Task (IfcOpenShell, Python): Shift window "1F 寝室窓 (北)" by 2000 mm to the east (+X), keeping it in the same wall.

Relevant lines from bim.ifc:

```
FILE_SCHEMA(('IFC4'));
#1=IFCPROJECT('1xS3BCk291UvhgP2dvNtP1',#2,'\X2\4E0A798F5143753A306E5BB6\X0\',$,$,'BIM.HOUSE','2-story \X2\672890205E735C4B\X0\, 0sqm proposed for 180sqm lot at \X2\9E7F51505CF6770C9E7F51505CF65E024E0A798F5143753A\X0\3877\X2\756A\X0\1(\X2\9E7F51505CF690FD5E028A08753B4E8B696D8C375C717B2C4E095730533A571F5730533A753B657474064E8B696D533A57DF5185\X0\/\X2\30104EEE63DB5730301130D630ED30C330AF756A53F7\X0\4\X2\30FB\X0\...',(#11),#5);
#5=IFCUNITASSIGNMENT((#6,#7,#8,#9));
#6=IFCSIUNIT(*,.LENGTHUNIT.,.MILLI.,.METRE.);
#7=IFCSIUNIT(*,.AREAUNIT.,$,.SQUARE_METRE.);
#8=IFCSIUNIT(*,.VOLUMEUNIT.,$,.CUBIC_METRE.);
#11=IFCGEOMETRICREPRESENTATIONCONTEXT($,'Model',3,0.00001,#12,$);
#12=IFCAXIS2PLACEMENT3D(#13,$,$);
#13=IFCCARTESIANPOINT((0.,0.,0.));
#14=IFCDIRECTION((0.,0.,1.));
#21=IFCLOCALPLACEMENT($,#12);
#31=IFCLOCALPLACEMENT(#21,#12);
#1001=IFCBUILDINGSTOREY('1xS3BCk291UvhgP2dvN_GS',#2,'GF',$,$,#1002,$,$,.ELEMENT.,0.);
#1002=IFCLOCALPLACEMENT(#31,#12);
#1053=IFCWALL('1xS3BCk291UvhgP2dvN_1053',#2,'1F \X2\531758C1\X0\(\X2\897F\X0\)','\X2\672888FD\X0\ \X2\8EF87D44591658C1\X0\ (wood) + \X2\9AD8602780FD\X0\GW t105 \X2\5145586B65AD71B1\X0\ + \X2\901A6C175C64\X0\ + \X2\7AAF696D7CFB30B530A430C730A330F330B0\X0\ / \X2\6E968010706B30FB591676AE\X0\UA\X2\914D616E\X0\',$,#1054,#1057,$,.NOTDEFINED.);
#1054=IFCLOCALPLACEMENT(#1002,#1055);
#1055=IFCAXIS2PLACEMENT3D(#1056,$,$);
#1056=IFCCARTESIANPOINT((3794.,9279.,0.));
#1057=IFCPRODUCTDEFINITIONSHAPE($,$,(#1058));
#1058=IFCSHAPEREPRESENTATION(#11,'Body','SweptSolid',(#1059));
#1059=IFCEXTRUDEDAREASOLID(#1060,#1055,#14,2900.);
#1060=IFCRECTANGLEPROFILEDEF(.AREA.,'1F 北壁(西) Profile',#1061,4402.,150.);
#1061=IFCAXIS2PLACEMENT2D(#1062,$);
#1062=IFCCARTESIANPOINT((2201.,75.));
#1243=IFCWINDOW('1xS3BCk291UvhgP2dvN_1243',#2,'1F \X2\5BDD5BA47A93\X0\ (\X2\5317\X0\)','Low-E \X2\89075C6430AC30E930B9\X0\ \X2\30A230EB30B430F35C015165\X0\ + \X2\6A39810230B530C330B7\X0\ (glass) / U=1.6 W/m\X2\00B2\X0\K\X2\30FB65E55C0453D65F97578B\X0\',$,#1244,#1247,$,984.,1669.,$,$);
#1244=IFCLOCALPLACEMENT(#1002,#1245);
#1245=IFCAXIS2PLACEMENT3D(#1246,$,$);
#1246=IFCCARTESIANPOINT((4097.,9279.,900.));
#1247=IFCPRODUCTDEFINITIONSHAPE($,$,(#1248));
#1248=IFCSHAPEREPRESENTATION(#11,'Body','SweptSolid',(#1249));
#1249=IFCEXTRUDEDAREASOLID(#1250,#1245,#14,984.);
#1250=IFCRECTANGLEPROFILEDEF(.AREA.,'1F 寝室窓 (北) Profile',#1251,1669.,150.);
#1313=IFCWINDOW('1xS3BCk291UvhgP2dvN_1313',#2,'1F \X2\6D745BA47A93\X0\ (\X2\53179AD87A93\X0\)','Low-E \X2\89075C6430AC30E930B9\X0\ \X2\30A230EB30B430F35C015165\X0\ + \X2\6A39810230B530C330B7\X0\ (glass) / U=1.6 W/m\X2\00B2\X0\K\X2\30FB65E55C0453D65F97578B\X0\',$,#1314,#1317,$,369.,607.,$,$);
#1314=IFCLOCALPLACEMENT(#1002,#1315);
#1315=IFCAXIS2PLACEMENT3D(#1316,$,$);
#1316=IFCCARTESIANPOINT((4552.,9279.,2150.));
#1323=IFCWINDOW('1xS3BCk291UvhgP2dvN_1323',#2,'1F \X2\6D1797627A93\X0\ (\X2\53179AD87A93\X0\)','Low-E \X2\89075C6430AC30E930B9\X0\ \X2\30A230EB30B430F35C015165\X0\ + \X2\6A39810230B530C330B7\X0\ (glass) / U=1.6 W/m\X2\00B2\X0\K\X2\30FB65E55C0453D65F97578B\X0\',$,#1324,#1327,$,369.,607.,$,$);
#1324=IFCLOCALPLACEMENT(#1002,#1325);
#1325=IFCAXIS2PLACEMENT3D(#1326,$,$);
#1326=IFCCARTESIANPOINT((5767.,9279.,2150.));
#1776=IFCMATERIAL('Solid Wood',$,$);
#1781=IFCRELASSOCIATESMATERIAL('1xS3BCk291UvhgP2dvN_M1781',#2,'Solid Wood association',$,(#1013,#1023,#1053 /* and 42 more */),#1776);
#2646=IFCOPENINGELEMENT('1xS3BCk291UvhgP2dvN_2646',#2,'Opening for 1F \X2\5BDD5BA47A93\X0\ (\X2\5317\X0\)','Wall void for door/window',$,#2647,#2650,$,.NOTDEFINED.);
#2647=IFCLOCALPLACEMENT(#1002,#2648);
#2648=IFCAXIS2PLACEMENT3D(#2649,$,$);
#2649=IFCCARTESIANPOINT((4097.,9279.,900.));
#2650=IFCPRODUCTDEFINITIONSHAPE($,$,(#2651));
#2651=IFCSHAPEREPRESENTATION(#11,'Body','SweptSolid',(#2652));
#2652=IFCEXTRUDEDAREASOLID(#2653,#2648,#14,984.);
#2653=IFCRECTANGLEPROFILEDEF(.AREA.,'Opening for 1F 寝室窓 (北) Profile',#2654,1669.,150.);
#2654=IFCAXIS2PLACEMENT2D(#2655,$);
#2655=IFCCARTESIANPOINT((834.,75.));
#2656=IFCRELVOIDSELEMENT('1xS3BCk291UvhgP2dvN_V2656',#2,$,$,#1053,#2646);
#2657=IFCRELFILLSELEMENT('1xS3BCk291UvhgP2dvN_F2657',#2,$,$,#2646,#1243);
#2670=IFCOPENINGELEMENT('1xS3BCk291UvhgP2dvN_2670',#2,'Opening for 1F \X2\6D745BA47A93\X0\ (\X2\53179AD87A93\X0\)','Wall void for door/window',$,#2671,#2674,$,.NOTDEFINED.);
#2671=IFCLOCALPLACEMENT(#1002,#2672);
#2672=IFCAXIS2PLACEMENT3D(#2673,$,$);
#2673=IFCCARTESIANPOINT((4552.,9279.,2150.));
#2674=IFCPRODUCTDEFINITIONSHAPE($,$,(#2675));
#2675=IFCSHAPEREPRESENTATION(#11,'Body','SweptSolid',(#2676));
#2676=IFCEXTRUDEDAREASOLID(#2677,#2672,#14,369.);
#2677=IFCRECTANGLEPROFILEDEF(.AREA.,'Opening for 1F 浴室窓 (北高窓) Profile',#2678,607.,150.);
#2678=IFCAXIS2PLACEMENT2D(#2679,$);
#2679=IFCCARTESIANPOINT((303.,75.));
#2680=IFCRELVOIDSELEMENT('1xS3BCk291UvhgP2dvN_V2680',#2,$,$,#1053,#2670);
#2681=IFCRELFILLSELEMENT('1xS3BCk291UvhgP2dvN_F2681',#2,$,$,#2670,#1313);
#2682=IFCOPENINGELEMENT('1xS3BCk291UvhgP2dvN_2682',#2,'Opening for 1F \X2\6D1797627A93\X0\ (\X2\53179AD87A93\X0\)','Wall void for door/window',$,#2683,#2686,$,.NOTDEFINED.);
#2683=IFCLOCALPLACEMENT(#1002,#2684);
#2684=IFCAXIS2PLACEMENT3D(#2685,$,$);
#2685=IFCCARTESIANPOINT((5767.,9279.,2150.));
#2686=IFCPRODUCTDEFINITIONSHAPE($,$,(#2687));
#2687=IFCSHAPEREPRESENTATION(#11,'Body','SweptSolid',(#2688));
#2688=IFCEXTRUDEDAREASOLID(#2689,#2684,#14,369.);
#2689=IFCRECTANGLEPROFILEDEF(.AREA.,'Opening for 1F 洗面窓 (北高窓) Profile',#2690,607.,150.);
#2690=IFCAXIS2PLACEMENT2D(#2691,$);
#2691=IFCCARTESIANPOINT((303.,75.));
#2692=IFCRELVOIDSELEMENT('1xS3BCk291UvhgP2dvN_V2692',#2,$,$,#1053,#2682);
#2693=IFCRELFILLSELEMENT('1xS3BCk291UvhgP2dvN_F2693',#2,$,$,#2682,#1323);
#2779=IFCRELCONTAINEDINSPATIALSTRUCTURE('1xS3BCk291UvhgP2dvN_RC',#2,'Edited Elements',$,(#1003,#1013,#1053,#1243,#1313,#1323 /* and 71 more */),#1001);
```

```python
import ifcopenshell
import ifcopenshell.api.geometry
import ifcopenshell.util.placement
import ifcopenshell.util.unit

model = ifcopenshell.open("bim.ifc")
unit_scale = ifcopenshell.util.unit.calculate_unit_scale(model)

window = model.by_guid("1xS3BCk291UvhgP2dvN_1243")
opening = window.FillsVoids[0].RelatingOpeningElement
wall = opening.VoidsElements[0].RelatingBuildingElement

wall_matrix = ifcopenshell.util.placement.get_local_placement(wall.ObjectPlacement)
shift = wall_matrix[:3, 0] * 2 / unit_scale
before = ifcopenshell.util.placement.get_local_placement(window.ObjectPlacement)[:3, 3].copy()

# The window is not placed relative to its opening, so move both.
for product in (opening, window):
    matrix = ifcopenshell.util.placement.get_local_placement(product.ObjectPlacement)
    matrix[:3, 3] += shift
    ifcopenshell.api.geometry.edit_object_placement(model, product=product, matrix=matrix, is_si=False)

after = ifcopenshell.util.placement.get_local_placement(window.ObjectPlacement)[:3, 3]
print("window moved by", (after - before).round(3) + 0.0)

model.write("bim_edited.ifc")
```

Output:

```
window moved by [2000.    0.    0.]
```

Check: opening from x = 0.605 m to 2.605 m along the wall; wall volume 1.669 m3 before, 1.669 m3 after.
